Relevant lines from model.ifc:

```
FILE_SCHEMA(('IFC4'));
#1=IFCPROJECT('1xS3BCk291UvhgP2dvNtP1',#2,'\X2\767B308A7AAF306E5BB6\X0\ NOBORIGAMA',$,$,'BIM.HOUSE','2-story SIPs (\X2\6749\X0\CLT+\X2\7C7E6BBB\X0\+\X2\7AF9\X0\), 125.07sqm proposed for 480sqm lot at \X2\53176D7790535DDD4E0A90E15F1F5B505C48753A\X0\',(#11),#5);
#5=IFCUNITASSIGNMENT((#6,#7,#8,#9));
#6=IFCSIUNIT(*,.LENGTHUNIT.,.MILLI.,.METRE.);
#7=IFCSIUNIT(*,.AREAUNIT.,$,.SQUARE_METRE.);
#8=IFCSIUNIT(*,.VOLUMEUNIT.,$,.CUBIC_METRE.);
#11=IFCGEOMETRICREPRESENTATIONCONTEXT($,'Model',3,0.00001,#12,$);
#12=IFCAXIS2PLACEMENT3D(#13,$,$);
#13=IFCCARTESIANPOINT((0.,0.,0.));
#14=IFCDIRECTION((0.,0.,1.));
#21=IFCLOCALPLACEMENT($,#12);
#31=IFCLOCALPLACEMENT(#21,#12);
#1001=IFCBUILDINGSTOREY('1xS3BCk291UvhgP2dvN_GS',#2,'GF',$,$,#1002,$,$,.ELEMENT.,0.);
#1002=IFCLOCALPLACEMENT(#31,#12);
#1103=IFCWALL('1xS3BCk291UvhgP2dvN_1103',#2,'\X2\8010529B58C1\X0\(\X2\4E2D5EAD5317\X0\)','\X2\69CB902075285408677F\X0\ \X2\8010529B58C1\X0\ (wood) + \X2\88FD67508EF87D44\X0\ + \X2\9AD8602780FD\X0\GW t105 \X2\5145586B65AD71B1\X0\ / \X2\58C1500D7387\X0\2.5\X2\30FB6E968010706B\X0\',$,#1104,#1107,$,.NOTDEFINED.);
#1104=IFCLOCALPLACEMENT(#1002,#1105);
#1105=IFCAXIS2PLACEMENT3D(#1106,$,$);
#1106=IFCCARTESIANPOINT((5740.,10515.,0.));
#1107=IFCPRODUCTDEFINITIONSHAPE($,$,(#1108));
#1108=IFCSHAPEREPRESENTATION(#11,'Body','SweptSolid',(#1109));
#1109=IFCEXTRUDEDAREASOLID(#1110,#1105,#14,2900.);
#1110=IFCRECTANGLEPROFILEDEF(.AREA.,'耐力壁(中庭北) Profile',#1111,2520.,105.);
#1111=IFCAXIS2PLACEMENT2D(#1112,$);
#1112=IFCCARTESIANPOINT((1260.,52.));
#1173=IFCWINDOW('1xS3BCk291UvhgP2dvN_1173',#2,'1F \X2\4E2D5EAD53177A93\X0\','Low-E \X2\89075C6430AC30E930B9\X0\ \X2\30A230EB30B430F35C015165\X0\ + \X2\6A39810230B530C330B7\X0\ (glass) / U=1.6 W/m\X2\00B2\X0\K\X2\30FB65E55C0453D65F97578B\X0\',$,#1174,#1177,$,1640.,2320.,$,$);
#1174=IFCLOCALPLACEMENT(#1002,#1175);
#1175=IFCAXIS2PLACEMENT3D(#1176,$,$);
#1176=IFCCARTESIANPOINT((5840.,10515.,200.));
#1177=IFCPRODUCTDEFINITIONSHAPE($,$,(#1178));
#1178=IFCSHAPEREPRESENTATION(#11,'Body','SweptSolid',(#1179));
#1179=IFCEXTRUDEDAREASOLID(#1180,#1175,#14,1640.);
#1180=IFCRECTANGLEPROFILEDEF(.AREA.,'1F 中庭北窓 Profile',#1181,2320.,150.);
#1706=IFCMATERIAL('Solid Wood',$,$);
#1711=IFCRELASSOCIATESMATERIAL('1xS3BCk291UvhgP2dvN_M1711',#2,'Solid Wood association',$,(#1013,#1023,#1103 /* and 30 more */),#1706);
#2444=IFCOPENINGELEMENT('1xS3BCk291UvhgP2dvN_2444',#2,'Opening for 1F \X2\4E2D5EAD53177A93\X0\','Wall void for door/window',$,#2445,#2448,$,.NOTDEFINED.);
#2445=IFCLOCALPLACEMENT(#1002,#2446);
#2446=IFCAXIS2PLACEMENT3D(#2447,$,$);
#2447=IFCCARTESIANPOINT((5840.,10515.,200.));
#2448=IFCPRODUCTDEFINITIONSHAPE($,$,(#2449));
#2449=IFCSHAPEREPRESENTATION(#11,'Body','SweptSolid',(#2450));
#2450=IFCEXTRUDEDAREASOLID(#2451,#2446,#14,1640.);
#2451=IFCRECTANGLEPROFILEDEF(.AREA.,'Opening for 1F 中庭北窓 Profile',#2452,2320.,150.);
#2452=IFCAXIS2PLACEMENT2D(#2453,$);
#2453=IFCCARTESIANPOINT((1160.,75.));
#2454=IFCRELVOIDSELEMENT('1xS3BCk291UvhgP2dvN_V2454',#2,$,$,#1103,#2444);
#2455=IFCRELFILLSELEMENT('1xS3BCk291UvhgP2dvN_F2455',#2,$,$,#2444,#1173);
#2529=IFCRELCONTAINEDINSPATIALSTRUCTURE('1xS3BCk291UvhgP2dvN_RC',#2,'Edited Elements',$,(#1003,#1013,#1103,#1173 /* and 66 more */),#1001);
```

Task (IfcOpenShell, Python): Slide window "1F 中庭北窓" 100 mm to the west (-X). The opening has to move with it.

```python
import ifcopenshell
import ifcopenshell.api.geometry
import ifcopenshell.util.placement

model = ifcopenshell.open("model.ifc")

window = model.by_guid("1xS3BCk291UvhgP2dvN_1173")
opening = window.FillsVoids[0].RelatingOpeningElement
wall = opening.VoidsElements[0].RelatingBuildingElement

wall_matrix = ifcopenshell.util.placement.get_local_placement(wall.ObjectPlacement)
shift = wall_matrix[:3, 0] * -100.0
before = ifcopenshell.util.placement.get_local_placement(window.ObjectPlacement)[:3, 3].copy()

# The window is not placed relative to its opening, so move both.
for product in (opening, window):
    matrix = ifcopenshell.util.placement.get_local_placement(product.ObjectPlacement)
    matrix[:3, 3] += shift
    ifcopenshell.api.geometry.edit_object_placement(model, product=product, matrix=matrix, is_si=False)

after = ifcopenshell.util.placement.get_local_placement(window.ObjectPlacement)[:3, 3]
print("window moved by", (after - before).round(3) + 0.0)

model.write("model_edited.ifc")
```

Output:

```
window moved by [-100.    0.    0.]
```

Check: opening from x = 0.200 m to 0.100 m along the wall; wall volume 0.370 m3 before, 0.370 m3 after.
